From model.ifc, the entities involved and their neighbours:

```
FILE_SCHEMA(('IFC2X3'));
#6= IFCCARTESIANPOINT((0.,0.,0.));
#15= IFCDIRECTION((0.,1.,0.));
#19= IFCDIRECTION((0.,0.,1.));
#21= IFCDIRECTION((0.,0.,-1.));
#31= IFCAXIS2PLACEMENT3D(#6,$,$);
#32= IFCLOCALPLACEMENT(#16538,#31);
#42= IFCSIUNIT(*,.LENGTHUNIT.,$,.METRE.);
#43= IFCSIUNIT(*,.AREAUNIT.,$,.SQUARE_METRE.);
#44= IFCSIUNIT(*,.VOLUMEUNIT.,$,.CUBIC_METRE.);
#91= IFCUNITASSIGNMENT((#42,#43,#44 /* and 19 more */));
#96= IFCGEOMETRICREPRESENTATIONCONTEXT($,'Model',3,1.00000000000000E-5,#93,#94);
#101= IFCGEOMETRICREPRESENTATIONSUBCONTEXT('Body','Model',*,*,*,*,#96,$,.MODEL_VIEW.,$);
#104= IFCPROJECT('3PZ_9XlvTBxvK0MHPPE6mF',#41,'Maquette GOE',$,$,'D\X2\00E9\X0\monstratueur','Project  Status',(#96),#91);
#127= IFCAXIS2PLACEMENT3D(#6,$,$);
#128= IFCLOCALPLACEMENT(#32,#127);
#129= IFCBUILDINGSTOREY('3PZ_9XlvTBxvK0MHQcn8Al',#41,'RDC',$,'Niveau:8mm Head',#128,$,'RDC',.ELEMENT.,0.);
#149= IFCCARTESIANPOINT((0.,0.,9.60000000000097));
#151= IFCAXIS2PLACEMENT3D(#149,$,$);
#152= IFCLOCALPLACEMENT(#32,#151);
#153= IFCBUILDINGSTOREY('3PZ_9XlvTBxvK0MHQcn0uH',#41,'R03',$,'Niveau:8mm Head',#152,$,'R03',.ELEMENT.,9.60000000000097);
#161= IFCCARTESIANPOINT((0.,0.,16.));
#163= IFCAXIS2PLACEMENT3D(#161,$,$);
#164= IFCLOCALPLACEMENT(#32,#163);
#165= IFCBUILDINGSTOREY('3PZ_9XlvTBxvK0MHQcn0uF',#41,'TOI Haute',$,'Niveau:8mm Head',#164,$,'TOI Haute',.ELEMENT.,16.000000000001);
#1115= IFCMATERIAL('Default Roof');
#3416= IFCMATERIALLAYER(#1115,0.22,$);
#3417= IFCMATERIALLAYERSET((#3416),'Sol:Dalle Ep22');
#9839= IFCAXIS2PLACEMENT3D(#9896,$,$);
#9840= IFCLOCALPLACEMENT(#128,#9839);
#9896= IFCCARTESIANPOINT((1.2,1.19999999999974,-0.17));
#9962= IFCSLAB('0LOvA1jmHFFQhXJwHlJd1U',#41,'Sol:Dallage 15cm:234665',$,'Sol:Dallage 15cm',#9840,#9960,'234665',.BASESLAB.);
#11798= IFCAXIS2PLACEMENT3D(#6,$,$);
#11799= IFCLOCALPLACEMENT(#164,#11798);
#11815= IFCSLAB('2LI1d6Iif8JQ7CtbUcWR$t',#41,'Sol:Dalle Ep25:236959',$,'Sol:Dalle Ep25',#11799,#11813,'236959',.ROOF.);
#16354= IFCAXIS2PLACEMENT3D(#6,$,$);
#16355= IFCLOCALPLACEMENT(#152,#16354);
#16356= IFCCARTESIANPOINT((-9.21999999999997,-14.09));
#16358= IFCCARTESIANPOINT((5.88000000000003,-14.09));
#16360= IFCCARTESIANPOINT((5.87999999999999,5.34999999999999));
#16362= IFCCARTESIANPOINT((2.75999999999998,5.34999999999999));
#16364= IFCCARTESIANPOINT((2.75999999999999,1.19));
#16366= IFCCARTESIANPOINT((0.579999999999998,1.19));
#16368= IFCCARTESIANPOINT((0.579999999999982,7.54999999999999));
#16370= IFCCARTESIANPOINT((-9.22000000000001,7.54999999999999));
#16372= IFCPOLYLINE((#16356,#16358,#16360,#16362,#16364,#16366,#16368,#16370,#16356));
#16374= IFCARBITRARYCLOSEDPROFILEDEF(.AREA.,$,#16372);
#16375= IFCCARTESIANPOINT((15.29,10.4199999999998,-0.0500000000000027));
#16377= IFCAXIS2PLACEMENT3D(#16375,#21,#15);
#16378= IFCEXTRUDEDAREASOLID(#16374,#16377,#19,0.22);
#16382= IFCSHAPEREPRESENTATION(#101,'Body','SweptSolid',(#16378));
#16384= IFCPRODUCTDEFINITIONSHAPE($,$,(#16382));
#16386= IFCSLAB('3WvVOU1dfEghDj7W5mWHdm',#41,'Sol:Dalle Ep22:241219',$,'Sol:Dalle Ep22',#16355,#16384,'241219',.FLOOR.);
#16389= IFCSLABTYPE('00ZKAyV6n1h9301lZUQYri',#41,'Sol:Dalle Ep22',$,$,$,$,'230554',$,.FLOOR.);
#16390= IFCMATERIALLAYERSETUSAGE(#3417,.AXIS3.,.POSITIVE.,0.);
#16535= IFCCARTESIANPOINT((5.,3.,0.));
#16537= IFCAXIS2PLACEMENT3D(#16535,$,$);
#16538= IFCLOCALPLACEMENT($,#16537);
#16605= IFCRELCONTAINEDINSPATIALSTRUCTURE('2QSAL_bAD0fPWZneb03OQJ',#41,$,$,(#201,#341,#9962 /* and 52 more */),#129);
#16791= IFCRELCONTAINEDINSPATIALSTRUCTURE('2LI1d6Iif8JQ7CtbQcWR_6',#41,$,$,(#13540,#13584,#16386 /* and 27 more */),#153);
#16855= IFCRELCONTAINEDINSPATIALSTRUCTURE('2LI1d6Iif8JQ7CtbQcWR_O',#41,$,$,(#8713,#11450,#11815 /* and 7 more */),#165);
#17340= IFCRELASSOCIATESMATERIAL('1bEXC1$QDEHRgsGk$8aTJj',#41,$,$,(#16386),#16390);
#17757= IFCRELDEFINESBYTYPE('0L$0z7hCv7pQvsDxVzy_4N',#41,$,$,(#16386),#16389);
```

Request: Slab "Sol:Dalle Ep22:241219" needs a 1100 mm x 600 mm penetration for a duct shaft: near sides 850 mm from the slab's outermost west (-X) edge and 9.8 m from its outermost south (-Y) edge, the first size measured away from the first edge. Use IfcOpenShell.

```python
import numpy as np
import ifcopenshell
import ifcopenshell.api.feature
import ifcopenshell.api.geometry
import ifcopenshell.api.root
import ifcopenshell.geom
import ifcopenshell.util.placement
import ifcopenshell.util.representation
import ifcopenshell.util.shape
import ifcopenshell.util.unit

model = ifcopenshell.open("model.ifc")
unit_scale = ifcopenshell.util.unit.calculate_unit_scale(model)
settings = ifcopenshell.geom.settings()


def volume(element):
    """Net volume in cubic metres, openings subtracted."""
    shape = ifcopenshell.geom.create_shape(settings, element)
    return ifcopenshell.util.shape.get_volume(shape.geometry)


slab = model.by_guid("3WvVOU1dfEghDj7W5mWHdm")
before = volume(slab)

# Extent in the slab's own axes, in metres. The edges named are its -X and -Y sides.
slab_shape = ifcopenshell.geom.create_shape(settings, slab)
vertices = ifcopenshell.util.shape.get_vertices(slab_shape.geometry)
x_min, y_min, bottom = vertices.min(axis=0)
top = vertices[:, 2].max()

opening = ifcopenshell.api.root.create_entity(model, ifc_class="IfcOpeningElement", name="Duct shaft opening")
context = ifcopenshell.util.representation.get_context(model, "Model", "Body", "MODEL_VIEW")
width, depth = 1.1, 0.6
outline = [(0.0, 0.0), (width, 0.0), (width, depth), (0.0, depth), (0.0, 0.0)]
# Overshoot both faces by 50 mm so the cut is clean.
shape = ifcopenshell.api.geometry.add_slab_representation(
    model, context=context, depth=top - bottom + 0.1, polyline=outline
)
ifcopenshell.api.geometry.assign_representation(model, product=opening, representation=shape)

matrix = ifcopenshell.util.placement.get_local_placement(slab.ObjectPlacement)
matrix[:, 3] = matrix @ np.append(np.array([x_min + 0.85, y_min + 9.8, bottom - 0.05]) / unit_scale, 1.0)
ifcopenshell.api.geometry.edit_object_placement(model, product=opening, matrix=matrix, is_si=False)
ifcopenshell.api.feature.add_feature(model, feature=opening, element=slab)

after = volume(slab)

print(f"slab volume {before:.3f} -> {after:.3f} m3")

model.write("model_rev.ifc")
```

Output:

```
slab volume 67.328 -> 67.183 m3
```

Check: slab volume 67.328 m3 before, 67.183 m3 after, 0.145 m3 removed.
